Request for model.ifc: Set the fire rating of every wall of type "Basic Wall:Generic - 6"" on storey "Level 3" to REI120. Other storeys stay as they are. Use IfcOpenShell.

First a look at what the model holds.

```python
import ifcopenshell
import ifcopenshell.util.element

model = ifcopenshell.open("model.ifc")
print(model.schema)
storey = next(s for s in model.by_type("IfcBuildingStorey") if s.Name == "Level 3")
walls = [e for e in ifcopenshell.util.element.get_decomposition(storey) if e.is_a("IfcWall")]
seen = {}
for e in walls:
    element_type = ifcopenshell.util.element.get_type(e)
    key = (element_type.Name if element_type != e and element_type else None, ifcopenshell.util.element.get_pset(e, "Pset_WallCommon", "FireRating"))
    seen[key] = seen.get(key, 0) + 1
for (name, value), count in sorted(seen.items(), key=str):
    print(count, "x", name, "|", value)
```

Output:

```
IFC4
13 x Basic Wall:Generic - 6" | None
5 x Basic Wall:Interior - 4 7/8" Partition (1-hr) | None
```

```python
import ifcopenshell
import ifcopenshell.api.pset
import ifcopenshell.util.element

model = ifcopenshell.open("model.ifc")

storey = next(s for s in model.by_type("IfcBuildingStorey") if s.Name == "Level 3")
walls = [e for e in ifcopenshell.util.element.get_decomposition(storey) if e.is_a("IfcWall")]

count = 0
for e in walls:
    element_type = ifcopenshell.util.element.get_type(e)
    if element_type in (None, e) or element_type.Name != 'Basic Wall:Generic - 6"':
        continue
    # add_pset returns the element's existing set when there is one.
    pset = ifcopenshell.api.pset.add_pset(model, product=e, name="Pset_WallCommon")
    ifcopenshell.api.pset.edit_pset(model, pset=pset, properties={"FireRating": "REI120"})
    count += 1

print(count, "walls updated")

model.write("model_edited.ifc")
```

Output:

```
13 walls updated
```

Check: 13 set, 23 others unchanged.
